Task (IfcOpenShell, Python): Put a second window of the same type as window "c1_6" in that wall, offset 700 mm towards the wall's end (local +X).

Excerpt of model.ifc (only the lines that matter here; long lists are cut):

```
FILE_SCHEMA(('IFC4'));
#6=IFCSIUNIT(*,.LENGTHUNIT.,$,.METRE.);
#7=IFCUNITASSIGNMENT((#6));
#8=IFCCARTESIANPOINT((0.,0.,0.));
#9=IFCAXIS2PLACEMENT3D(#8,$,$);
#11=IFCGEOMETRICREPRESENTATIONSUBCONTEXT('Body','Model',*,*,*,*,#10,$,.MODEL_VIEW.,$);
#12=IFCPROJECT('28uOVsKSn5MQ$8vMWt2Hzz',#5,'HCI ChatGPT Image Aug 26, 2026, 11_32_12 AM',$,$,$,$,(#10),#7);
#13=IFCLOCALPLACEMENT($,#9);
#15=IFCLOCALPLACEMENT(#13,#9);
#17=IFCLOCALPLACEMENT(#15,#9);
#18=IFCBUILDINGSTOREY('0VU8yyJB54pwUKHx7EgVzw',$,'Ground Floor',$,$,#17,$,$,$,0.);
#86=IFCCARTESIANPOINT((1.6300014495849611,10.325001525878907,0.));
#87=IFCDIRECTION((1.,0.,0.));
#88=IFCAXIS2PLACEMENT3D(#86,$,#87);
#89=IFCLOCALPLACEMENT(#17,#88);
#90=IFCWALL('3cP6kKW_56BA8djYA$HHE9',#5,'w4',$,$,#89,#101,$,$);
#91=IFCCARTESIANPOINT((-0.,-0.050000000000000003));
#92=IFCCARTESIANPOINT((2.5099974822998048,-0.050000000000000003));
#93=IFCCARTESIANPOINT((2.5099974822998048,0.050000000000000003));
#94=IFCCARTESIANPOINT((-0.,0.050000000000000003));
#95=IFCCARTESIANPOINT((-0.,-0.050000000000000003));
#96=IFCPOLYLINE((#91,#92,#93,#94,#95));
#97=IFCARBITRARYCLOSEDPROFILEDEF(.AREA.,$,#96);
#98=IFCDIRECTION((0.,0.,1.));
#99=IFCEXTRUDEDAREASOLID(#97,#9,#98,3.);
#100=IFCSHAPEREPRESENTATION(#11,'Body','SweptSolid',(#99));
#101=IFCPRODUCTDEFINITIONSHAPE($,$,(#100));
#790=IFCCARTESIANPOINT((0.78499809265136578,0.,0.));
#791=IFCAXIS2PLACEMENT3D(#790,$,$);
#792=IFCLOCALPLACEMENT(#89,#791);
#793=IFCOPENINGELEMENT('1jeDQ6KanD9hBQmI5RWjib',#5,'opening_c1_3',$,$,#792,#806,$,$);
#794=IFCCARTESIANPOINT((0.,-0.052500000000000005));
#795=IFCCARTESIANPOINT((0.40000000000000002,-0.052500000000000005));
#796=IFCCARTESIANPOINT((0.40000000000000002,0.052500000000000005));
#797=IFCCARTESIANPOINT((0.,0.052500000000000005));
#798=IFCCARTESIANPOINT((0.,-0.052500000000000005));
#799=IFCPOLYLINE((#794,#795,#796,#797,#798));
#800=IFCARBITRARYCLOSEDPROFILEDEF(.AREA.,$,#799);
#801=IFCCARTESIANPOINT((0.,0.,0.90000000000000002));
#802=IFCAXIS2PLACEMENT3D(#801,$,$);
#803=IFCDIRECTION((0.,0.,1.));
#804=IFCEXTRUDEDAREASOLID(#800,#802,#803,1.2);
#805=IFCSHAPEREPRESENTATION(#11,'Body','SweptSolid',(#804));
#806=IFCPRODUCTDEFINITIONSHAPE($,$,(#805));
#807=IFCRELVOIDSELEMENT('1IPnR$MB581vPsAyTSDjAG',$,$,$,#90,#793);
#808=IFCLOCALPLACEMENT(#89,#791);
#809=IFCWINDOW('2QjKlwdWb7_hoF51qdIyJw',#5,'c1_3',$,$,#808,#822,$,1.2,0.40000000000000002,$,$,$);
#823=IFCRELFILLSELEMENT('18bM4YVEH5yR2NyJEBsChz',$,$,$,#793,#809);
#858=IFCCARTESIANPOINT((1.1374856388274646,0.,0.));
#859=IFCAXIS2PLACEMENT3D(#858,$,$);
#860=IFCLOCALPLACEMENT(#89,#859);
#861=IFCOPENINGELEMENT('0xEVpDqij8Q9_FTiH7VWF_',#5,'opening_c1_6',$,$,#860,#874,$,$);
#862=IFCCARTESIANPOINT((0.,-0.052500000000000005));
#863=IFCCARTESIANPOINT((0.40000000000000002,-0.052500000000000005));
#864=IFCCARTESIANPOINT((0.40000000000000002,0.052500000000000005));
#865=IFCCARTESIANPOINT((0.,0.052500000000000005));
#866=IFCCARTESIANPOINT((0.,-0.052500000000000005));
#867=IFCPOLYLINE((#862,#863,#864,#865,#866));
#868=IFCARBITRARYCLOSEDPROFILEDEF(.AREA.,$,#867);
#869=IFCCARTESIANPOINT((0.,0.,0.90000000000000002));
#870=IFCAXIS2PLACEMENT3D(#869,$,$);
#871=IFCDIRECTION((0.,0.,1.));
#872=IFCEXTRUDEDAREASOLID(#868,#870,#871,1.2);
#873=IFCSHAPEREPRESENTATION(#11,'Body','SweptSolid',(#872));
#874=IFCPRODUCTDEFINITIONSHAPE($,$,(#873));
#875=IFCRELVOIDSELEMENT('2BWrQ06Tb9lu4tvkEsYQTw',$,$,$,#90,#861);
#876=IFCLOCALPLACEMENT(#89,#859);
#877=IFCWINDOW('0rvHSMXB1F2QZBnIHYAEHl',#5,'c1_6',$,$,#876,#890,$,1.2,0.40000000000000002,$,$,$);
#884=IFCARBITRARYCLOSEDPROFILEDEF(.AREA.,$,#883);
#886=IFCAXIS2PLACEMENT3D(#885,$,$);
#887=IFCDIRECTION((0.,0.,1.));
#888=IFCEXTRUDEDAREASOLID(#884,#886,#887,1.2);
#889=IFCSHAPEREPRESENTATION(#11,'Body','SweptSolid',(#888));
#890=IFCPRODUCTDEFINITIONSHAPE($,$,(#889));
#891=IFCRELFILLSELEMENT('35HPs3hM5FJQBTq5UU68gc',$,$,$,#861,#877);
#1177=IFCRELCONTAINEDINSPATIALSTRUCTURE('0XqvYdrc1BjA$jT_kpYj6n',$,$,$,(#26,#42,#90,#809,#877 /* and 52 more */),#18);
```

```python
import ifcopenshell
import ifcopenshell.api.feature
import ifcopenshell.api.geometry
import ifcopenshell.api.root
import ifcopenshell.geom
import ifcopenshell.util.element
import ifcopenshell.util.placement
import ifcopenshell.util.shape

model = ifcopenshell.open("model.ifc")
settings = ifcopenshell.geom.settings()


def volume(element):
    """Net volume in cubic metres, openings subtracted."""
    shape = ifcopenshell.geom.create_shape(settings, element)
    return ifcopenshell.util.shape.get_volume(shape.geometry)


window = model.by_guid("0rvHSMXB1F2QZBnIHYAEHl")
opening = window.FillsVoids[0].RelatingOpeningElement
wall = opening.VoidsElements[0].RelatingBuildingElement
before = volume(wall)
shift = ifcopenshell.util.placement.get_local_placement(wall.ObjectPlacement)[:3, 0] * 0.7

# copy_class copies the void relationship, type, container and properties, but no geometry.
new_opening = ifcopenshell.api.root.copy_class(model, product=opening)
new_opening.Representation = ifcopenshell.util.element.copy_deep(
    model, opening.Representation, exclude=["IfcGeometricRepresentationContext", "IfcRepresentationMap"]
)
new_window = ifcopenshell.api.root.copy_class(model, product=window)
new_window.Representation = ifcopenshell.util.element.copy_deep(
    model, window.Representation, exclude=["IfcGeometricRepresentationContext", "IfcRepresentationMap"]
)
ifcopenshell.api.feature.add_filling(model, opening=new_opening, element=new_window)

for old, new in ((opening, new_opening), (window, new_window)):
    matrix = ifcopenshell.util.placement.get_local_placement(old.ObjectPlacement)
    matrix[:3, 3] += shift
    ifcopenshell.api.geometry.edit_object_placement(model, product=new, matrix=matrix, is_si=False)

after = volume(wall)

print(f"wall volume {before:.3f} -> {after:.3f} m3")

model.write("model_updated.ifc")
```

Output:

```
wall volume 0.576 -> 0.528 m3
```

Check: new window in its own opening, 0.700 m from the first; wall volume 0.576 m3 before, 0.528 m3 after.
